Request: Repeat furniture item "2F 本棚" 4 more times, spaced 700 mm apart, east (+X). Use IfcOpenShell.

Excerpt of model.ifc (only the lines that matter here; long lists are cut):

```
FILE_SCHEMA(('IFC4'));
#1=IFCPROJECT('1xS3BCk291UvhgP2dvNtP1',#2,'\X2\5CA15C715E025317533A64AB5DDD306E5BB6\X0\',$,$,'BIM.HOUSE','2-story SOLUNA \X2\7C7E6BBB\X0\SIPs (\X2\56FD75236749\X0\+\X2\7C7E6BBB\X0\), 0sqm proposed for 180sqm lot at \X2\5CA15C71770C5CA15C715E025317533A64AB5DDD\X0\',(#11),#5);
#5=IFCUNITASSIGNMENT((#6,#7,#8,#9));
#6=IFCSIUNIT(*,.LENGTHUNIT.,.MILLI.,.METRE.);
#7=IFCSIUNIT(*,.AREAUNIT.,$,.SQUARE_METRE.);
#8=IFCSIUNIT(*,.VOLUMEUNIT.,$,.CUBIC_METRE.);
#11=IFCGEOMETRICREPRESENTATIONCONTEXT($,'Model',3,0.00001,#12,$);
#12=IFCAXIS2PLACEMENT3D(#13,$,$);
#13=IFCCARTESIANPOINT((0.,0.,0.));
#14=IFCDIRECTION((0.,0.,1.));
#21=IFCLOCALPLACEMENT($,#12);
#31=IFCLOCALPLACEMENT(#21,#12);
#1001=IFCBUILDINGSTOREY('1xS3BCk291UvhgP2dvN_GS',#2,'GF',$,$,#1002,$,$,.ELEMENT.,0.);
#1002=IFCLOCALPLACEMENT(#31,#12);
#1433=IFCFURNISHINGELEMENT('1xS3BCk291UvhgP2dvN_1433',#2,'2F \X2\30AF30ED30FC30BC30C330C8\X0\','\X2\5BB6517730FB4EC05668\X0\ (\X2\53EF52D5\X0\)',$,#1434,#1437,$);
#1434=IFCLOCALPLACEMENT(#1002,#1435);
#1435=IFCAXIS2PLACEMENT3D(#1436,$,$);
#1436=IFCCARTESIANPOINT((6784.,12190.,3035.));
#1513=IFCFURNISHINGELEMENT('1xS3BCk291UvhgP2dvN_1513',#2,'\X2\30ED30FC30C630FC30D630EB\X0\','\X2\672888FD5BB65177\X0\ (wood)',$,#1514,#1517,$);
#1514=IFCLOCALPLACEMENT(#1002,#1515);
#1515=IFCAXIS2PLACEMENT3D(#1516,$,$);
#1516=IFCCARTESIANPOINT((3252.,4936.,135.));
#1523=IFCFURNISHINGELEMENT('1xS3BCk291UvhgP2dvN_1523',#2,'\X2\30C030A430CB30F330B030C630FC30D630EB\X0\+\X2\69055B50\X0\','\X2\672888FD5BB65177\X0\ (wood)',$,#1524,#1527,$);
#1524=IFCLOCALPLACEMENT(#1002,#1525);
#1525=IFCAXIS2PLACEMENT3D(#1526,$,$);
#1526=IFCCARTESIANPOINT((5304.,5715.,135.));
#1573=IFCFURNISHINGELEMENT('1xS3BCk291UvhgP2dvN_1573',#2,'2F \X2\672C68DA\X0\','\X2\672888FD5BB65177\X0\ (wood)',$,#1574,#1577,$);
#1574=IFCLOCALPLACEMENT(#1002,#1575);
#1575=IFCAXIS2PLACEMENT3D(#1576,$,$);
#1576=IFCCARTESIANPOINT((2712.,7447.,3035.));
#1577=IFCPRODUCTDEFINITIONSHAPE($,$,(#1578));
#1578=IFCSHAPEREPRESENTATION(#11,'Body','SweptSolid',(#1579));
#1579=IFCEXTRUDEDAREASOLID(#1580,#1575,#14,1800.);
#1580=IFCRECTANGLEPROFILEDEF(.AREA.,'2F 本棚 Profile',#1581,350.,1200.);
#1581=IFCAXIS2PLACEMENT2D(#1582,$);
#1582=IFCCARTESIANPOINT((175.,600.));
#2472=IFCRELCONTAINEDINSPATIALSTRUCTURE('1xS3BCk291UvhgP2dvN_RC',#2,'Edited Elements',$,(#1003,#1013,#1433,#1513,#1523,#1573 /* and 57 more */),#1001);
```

```python
import numpy as np
import ifcopenshell
import ifcopenshell.api.geometry
import ifcopenshell.api.root
import ifcopenshell.util.element
import ifcopenshell.util.placement
import ifcopenshell.util.unit

model = ifcopenshell.open("model.ifc")
unit_scale = ifcopenshell.util.unit.calculate_unit_scale(model)


def reuse_history(source, copy):
    """copy_class also copies each property set's owner history, people and application; keep the originals."""
    for rel in copy.IsDefinedBy:
        if rel.is_a("IfcRelDefinesByProperties") and (history := rel.RelatingPropertyDefinition.OwnerHistory):
            rel.RelatingPropertyDefinition.OwnerHistory = source.OwnerHistory
            ifcopenshell.util.element.remove_deep2(model, history)


source = model.by_guid("1xS3BCk291UvhgP2dvN_1573")
base = ifcopenshell.util.placement.get_local_placement(source.ObjectPlacement)
step = np.array([1.0, 0.0, 0.0]) * 0.7 / unit_scale

for i in range(1, 5):
    copy = ifcopenshell.api.root.copy_class(model, product=source)
    copy.Representation = ifcopenshell.util.element.copy_deep(
        model, source.Representation, exclude=["IfcGeometricRepresentationContext", "IfcRepresentationMap"]
    )
    reuse_history(source, copy)
    matrix = base.copy()
    matrix[:3, 3] += i * step
    print("added at", matrix[:3, 3].round(3) + 0.0)
    ifcopenshell.api.geometry.edit_object_placement(model, product=copy, matrix=matrix, is_si=False)

model.write("model_v2.ifc")
```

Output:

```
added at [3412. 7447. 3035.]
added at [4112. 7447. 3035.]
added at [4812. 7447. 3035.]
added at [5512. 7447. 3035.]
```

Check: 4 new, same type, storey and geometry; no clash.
